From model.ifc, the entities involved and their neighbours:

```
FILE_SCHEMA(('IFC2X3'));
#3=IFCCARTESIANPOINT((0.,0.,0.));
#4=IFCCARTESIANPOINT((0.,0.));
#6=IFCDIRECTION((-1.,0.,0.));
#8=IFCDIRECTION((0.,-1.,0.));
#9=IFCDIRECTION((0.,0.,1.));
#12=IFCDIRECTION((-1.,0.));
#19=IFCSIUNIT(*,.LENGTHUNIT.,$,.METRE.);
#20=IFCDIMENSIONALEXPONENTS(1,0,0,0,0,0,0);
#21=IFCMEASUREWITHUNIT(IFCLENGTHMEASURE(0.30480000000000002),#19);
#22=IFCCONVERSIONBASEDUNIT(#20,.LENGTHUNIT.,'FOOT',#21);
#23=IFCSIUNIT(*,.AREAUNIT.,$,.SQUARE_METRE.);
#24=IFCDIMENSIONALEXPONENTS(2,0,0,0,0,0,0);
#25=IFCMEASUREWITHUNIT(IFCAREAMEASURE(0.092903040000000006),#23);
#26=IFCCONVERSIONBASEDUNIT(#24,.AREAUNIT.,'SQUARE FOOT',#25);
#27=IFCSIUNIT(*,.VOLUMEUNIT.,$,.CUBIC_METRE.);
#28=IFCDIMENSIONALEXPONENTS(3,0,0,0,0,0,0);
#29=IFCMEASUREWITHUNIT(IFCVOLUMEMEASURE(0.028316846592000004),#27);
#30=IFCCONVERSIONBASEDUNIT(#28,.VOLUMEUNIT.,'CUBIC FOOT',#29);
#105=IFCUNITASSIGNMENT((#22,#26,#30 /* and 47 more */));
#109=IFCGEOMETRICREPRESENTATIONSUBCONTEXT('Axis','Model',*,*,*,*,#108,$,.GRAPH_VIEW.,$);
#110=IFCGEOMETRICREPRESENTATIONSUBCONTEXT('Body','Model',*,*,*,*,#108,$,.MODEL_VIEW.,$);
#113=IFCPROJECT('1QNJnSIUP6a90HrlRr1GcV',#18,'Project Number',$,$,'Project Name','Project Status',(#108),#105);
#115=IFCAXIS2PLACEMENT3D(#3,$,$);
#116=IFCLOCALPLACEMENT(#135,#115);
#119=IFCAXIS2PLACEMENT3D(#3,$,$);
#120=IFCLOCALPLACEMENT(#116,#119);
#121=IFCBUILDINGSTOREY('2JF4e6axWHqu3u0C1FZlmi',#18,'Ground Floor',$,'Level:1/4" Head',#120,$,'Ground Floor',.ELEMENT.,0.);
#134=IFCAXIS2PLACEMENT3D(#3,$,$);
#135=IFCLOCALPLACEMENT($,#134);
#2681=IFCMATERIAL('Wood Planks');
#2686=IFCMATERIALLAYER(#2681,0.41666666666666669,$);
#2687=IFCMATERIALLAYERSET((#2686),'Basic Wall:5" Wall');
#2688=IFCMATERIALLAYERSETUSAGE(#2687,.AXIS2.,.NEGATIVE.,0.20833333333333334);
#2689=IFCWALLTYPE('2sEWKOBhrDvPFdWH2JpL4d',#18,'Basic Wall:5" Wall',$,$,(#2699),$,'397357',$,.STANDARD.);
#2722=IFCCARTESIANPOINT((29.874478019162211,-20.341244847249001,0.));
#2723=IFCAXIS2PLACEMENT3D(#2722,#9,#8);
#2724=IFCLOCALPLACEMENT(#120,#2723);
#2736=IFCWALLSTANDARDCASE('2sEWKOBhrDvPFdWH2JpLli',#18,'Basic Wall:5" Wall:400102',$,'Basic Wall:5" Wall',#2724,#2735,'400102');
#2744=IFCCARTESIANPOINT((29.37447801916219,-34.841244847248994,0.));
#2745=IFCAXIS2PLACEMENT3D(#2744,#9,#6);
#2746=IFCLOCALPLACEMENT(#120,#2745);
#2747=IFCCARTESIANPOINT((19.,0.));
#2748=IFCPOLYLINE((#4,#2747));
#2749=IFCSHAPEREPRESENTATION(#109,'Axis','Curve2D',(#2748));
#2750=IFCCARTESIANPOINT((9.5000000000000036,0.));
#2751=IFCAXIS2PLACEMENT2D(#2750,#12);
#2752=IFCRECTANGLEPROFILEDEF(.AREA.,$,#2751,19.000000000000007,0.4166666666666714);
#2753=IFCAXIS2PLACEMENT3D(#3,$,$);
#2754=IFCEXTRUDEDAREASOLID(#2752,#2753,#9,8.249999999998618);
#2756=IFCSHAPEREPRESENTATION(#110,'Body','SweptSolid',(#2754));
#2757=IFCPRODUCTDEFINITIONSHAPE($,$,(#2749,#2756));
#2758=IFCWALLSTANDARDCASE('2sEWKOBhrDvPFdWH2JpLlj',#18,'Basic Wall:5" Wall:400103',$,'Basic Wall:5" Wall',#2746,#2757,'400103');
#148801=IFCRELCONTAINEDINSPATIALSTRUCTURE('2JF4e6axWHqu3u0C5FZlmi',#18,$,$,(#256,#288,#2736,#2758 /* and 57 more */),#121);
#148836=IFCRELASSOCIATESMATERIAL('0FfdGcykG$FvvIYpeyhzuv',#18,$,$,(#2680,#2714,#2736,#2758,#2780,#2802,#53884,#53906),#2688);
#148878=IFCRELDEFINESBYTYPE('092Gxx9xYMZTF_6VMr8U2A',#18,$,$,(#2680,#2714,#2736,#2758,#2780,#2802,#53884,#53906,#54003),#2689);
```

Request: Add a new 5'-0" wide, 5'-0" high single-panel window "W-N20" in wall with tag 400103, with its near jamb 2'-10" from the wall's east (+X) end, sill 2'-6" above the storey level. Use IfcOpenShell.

```python
import numpy as np
import ifcopenshell
import ifcopenshell.api.feature
import ifcopenshell.api.geometry
import ifcopenshell.api.root
import ifcopenshell.api.spatial
import ifcopenshell.api.type
import ifcopenshell.geom
import ifcopenshell.util.element
import ifcopenshell.util.placement
import ifcopenshell.util.representation
import ifcopenshell.util.shape
import ifcopenshell.util.unit

model = ifcopenshell.open("model.ifc")
unit_scale = ifcopenshell.util.unit.calculate_unit_scale(model)
settings = ifcopenshell.geom.settings()


def volume(element):
    """Net volume in cubic metres, openings subtracted."""
    shape = ifcopenshell.geom.create_shape(settings, element)
    return ifcopenshell.util.shape.get_volume(shape.geometry)


wall = model.by_id(2758)
storey = ifcopenshell.util.element.get_container(wall, ifc_class="IfcBuildingStorey")
context = ifcopenshell.util.representation.get_context(model, "Model", "Body", "MODEL_VIEW")
before = volume(wall)

width, height, from_end, sill = 1.524, 1.524, 0.8636, 0.762  # metres

# The wall runs along its own X axis, and the end named is its -X end.
wall_shape = ifcopenshell.geom.create_shape(settings, wall)
x, y, z = ifcopenshell.util.shape.get_vertices(wall_shape.geometry).T
start = x.min() + from_end
face, thickness = float(y.min()), float(y.max() - y.min())
wall_matrix = ifcopenshell.util.placement.get_local_placement(wall.ObjectPlacement)
level = ifcopenshell.util.placement.get_local_placement(storey.ObjectPlacement)[2, 3]


def in_wall(x, y):
    """Placement at x, y metres in the wall's axes, at sill height."""
    matrix = wall_matrix.copy()
    matrix[:, 3] = wall_matrix @ np.array([x / unit_scale, y / unit_scale, 0.0, 1.0])
    matrix[2, 3] = level + sill / unit_scale
    return matrix


# Opening: a box that overshoots both wall faces by 50 mm.
opening = ifcopenshell.api.root.create_entity(model, ifc_class="IfcOpeningElement")
box = ifcopenshell.api.geometry.add_wall_representation(
    model, context=context, length=width, height=height, thickness=thickness + 0.1
)
ifcopenshell.api.geometry.assign_representation(model, product=opening, representation=box)
ifcopenshell.api.geometry.edit_object_placement(model, product=opening, matrix=in_wall(start, face - 0.05), is_si=False)
ifcopenshell.api.feature.add_feature(model, feature=opening, element=wall)

window = ifcopenshell.api.root.create_entity(model, ifc_class="IfcWindow", name="W-N20")
window.OverallWidth, window.OverallHeight = width / unit_scale, height / unit_scale
body = ifcopenshell.api.geometry.add_window_representation(
    model,
    context=context,
    overall_width=window.OverallWidth,
    overall_height=window.OverallHeight,
    partition_type="SINGLE_PANEL",
)
ifcopenshell.api.geometry.assign_representation(model, product=window, representation=body)
ifcopenshell.api.spatial.assign_container(model, products=[window], relating_structure=storey)
fills = ifcopenshell.api.feature.add_filling(model, opening=opening, element=window)
fills.OwnerHistory = window.OwnerHistory  # required in IFC2X3

# IFC2X3 keeps the operation on the window style.
style = ifcopenshell.api.root.create_entity(model, ifc_class="IfcWindowStyle", name="W-N20")
style.OperationType, style.ConstructionType = "SINGLE_PANEL", "NOTDEFINED"
style.ParameterTakesPrecedence = style.Sizeable = False
ifcopenshell.api.type.assign_type(model, related_objects=[window], relating_type=style)

# Centre the window in the wall's thickness.
ifcopenshell.api.geometry.edit_object_placement(model, product=window, matrix=in_wall(start, face), is_si=False)
window_shape = ifcopenshell.geom.create_shape(settings, window)
depth = ifcopenshell.util.shape.get_vertices(window_shape.geometry)[:, 1]
offset = face + thickness / 2 - (depth.min() + depth.max()) / 2
ifcopenshell.api.geometry.edit_object_placement(model, product=window, matrix=in_wall(start, offset), is_si=False)

after = volume(wall)

print(f"wall volume {before:.3f} -> {after:.3f} m3")

model.write("model_updated.ifc")
```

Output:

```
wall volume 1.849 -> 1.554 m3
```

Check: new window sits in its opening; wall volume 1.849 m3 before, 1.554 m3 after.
